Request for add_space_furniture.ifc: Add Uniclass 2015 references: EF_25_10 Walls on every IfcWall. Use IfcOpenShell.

First a look at what the model holds.

```python
import ifcopenshell

model = ifcopenshell.open("add_space_furniture.ifc")
print(model.schema)
print("classifications:", [c.Name for c in model.by_type("IfcClassification")])
for ifc_class in ("IfcDoor", "IfcRoof", "IfcStair", "IfcWall", "IfcWindow"):
    print(ifc_class, len(model.by_type(ifc_class)))
```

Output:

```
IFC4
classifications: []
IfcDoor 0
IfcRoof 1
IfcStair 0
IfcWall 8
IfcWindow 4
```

```python
import ifcopenshell
import ifcopenshell.api.classification

model = ifcopenshell.open("add_space_furniture.ifc")

system = ifcopenshell.api.classification.add_classification(model, classification="Uniclass 2015")

codes = {
    "IfcWall": ("EF_25_10", "Walls"),
}
for ifc_class, (code, name) in codes.items():
    products = model.by_type(ifc_class)
    ifcopenshell.api.classification.add_reference(
        model, products=products, classification=system, identification=code, name=name
    )
    print(code, len(products))

model.write("add_space_furniture_updated.ifc")
```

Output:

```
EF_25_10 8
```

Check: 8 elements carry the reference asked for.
